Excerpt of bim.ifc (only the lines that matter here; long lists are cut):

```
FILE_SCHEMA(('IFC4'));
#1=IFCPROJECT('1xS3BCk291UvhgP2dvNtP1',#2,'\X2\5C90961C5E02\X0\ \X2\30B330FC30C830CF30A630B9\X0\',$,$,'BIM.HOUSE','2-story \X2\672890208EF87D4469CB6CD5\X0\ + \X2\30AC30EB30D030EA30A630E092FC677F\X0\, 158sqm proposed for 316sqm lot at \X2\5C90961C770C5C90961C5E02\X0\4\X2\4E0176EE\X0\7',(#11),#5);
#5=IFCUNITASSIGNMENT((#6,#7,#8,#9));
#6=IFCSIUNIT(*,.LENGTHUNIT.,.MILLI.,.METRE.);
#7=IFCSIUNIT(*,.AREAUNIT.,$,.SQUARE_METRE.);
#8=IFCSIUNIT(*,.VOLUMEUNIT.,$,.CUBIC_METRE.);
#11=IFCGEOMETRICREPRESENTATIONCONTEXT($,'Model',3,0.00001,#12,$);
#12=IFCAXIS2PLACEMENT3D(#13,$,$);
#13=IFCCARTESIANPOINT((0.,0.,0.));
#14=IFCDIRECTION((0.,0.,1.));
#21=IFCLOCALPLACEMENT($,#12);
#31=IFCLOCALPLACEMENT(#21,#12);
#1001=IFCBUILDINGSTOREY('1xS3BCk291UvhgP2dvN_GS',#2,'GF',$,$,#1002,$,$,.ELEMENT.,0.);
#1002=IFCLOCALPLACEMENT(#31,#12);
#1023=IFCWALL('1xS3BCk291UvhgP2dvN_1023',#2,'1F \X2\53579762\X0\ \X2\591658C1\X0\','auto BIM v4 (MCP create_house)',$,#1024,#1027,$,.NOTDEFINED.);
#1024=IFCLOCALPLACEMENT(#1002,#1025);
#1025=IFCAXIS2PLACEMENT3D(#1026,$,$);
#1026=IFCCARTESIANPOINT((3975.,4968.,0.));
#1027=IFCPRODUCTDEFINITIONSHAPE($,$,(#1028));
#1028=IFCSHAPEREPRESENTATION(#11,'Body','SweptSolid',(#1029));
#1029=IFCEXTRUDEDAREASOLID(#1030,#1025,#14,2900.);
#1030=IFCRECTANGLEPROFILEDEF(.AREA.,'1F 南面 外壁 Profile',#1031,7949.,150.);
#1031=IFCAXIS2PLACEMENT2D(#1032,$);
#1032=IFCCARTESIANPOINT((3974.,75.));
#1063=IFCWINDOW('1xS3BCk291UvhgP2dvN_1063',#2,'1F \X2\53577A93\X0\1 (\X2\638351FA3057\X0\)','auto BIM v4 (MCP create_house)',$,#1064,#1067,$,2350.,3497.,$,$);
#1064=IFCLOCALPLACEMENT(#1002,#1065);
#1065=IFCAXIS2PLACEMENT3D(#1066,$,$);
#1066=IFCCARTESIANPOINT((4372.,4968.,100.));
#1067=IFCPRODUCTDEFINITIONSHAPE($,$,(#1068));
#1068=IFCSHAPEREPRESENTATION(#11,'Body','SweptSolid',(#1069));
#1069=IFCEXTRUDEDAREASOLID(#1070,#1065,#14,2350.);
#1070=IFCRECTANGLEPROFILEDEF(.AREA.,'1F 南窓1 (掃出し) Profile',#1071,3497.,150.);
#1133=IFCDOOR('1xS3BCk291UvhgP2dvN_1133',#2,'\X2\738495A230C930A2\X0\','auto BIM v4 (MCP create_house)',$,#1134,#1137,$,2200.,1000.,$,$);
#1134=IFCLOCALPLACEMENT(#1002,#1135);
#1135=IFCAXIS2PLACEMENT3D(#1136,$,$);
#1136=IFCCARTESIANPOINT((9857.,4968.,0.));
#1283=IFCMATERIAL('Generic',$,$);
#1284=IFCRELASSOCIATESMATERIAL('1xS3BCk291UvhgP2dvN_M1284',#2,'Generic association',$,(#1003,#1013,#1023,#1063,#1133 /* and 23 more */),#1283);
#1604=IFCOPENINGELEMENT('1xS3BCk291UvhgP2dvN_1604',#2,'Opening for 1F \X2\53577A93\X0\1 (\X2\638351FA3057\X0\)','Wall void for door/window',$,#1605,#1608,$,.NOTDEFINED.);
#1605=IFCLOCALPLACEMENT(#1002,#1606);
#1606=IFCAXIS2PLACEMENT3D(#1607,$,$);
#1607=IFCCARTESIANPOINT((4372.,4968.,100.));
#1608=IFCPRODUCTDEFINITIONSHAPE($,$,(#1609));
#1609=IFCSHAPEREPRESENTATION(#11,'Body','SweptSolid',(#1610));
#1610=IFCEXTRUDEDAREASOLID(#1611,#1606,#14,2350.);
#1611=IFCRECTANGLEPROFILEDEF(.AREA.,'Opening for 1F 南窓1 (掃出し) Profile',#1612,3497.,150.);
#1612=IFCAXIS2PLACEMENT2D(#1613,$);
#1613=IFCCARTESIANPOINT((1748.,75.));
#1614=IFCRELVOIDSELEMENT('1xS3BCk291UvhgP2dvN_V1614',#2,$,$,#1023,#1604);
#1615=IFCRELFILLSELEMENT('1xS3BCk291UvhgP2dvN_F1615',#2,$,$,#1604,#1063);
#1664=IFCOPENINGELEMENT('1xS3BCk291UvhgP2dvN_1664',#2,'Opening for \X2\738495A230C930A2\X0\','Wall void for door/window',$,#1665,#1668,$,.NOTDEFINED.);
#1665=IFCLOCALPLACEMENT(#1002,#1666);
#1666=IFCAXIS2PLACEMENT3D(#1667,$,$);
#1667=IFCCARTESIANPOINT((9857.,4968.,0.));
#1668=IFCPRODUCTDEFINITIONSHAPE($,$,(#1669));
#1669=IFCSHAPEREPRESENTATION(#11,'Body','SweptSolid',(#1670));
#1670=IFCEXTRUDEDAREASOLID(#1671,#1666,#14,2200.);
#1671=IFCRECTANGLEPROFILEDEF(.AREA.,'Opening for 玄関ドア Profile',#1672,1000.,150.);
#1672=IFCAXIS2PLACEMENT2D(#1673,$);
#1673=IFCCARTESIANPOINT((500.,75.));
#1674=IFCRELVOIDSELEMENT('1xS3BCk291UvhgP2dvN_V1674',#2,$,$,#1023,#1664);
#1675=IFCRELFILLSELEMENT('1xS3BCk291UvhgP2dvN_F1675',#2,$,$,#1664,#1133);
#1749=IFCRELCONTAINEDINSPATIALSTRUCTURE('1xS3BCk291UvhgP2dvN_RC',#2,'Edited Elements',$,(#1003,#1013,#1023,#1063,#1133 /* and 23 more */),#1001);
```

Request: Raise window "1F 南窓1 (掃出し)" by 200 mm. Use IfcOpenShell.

```python
import numpy as np
import ifcopenshell
import ifcopenshell.api.geometry
import ifcopenshell.util.placement
import ifcopenshell.util.unit

model = ifcopenshell.open("bim.ifc")
unit_scale = ifcopenshell.util.unit.calculate_unit_scale(model)

window = model.by_guid("1xS3BCk291UvhgP2dvN_1063")
opening = window.FillsVoids[0].RelatingOpeningElement
dz = 200.0

shift = np.array([0.0, 0.0, dz])
# The window is not placed relative to its opening, so move both.
for product in (opening, window):
    matrix = ifcopenshell.util.placement.get_local_placement(product.ObjectPlacement)
    matrix[:3, 3] += shift
    ifcopenshell.api.geometry.edit_object_placement(model, product=product, matrix=matrix, is_si=False)

print(f"moved by {dz * unit_scale:+.3f} m")

model.write("bim_edited.ifc")
```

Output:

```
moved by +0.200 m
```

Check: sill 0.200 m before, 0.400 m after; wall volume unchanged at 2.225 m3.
